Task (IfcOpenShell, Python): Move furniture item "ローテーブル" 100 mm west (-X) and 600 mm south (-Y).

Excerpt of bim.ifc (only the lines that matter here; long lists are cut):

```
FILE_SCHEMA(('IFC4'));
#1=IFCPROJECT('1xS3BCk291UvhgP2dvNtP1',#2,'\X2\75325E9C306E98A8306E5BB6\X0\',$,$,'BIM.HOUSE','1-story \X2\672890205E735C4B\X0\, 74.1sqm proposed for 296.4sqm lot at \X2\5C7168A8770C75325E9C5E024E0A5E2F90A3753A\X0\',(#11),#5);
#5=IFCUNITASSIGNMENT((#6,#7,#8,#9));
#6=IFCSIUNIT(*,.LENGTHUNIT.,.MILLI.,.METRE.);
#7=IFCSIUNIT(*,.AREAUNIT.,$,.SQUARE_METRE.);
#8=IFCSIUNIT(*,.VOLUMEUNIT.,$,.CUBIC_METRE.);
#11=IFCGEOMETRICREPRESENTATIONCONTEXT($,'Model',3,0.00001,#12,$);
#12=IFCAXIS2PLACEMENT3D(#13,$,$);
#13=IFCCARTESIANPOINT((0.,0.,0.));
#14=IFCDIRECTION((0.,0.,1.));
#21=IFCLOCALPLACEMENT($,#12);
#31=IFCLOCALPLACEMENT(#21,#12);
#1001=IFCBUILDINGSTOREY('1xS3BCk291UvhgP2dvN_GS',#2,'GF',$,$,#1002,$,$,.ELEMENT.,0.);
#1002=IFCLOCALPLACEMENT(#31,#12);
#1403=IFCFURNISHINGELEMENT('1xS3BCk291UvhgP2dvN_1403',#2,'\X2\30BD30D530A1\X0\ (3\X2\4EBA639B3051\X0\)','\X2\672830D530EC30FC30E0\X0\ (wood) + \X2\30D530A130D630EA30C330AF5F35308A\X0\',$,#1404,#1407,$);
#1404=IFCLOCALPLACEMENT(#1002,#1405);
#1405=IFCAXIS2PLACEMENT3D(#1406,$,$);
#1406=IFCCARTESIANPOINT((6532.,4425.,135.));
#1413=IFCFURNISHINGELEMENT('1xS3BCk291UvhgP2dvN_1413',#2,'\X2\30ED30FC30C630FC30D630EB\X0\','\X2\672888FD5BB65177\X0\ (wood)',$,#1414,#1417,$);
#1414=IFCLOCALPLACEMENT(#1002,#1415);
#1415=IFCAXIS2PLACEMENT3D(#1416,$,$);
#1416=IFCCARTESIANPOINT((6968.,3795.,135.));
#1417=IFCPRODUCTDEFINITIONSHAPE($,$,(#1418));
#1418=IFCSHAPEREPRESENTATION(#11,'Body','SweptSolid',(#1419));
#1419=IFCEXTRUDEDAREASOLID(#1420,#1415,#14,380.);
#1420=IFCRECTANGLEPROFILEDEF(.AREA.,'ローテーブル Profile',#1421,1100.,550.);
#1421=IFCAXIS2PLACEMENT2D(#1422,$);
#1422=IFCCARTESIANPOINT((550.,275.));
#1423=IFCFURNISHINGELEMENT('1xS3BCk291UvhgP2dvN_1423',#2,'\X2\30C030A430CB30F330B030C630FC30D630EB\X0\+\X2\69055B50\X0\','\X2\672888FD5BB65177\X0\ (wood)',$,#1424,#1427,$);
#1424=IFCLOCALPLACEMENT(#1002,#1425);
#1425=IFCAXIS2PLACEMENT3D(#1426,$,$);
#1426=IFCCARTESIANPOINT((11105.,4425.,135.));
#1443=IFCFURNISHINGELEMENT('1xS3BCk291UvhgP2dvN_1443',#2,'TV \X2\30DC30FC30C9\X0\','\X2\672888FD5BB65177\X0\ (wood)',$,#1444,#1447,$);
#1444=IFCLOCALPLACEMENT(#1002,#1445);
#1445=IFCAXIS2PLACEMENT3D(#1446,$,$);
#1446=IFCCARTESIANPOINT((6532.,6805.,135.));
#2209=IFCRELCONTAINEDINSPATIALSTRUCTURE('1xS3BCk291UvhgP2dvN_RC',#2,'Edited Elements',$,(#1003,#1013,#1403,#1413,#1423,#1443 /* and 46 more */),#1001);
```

```python
import ifcopenshell
import ifcopenshell.api.geometry
import ifcopenshell.util.placement
import ifcopenshell.util.unit

model = ifcopenshell.open("bim.ifc")
unit_scale = ifcopenshell.util.unit.calculate_unit_scale(model)

item = model.by_guid("1xS3BCk291UvhgP2dvN_1413")
matrix = ifcopenshell.util.placement.get_local_placement(item.ObjectPlacement)
matrix[0, 3] -= 0.1 / unit_scale
matrix[1, 3] -= 0.6 / unit_scale
ifcopenshell.api.geometry.edit_object_placement(model, product=item, matrix=matrix, is_si=False)

print(ifcopenshell.util.placement.get_local_placement(item.ObjectPlacement).round(3) + 0.0)

model.write("bim_updated.ifc")
```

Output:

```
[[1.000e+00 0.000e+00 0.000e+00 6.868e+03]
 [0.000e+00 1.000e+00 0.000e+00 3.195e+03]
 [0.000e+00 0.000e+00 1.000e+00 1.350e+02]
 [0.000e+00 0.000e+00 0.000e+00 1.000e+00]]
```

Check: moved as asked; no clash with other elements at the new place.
